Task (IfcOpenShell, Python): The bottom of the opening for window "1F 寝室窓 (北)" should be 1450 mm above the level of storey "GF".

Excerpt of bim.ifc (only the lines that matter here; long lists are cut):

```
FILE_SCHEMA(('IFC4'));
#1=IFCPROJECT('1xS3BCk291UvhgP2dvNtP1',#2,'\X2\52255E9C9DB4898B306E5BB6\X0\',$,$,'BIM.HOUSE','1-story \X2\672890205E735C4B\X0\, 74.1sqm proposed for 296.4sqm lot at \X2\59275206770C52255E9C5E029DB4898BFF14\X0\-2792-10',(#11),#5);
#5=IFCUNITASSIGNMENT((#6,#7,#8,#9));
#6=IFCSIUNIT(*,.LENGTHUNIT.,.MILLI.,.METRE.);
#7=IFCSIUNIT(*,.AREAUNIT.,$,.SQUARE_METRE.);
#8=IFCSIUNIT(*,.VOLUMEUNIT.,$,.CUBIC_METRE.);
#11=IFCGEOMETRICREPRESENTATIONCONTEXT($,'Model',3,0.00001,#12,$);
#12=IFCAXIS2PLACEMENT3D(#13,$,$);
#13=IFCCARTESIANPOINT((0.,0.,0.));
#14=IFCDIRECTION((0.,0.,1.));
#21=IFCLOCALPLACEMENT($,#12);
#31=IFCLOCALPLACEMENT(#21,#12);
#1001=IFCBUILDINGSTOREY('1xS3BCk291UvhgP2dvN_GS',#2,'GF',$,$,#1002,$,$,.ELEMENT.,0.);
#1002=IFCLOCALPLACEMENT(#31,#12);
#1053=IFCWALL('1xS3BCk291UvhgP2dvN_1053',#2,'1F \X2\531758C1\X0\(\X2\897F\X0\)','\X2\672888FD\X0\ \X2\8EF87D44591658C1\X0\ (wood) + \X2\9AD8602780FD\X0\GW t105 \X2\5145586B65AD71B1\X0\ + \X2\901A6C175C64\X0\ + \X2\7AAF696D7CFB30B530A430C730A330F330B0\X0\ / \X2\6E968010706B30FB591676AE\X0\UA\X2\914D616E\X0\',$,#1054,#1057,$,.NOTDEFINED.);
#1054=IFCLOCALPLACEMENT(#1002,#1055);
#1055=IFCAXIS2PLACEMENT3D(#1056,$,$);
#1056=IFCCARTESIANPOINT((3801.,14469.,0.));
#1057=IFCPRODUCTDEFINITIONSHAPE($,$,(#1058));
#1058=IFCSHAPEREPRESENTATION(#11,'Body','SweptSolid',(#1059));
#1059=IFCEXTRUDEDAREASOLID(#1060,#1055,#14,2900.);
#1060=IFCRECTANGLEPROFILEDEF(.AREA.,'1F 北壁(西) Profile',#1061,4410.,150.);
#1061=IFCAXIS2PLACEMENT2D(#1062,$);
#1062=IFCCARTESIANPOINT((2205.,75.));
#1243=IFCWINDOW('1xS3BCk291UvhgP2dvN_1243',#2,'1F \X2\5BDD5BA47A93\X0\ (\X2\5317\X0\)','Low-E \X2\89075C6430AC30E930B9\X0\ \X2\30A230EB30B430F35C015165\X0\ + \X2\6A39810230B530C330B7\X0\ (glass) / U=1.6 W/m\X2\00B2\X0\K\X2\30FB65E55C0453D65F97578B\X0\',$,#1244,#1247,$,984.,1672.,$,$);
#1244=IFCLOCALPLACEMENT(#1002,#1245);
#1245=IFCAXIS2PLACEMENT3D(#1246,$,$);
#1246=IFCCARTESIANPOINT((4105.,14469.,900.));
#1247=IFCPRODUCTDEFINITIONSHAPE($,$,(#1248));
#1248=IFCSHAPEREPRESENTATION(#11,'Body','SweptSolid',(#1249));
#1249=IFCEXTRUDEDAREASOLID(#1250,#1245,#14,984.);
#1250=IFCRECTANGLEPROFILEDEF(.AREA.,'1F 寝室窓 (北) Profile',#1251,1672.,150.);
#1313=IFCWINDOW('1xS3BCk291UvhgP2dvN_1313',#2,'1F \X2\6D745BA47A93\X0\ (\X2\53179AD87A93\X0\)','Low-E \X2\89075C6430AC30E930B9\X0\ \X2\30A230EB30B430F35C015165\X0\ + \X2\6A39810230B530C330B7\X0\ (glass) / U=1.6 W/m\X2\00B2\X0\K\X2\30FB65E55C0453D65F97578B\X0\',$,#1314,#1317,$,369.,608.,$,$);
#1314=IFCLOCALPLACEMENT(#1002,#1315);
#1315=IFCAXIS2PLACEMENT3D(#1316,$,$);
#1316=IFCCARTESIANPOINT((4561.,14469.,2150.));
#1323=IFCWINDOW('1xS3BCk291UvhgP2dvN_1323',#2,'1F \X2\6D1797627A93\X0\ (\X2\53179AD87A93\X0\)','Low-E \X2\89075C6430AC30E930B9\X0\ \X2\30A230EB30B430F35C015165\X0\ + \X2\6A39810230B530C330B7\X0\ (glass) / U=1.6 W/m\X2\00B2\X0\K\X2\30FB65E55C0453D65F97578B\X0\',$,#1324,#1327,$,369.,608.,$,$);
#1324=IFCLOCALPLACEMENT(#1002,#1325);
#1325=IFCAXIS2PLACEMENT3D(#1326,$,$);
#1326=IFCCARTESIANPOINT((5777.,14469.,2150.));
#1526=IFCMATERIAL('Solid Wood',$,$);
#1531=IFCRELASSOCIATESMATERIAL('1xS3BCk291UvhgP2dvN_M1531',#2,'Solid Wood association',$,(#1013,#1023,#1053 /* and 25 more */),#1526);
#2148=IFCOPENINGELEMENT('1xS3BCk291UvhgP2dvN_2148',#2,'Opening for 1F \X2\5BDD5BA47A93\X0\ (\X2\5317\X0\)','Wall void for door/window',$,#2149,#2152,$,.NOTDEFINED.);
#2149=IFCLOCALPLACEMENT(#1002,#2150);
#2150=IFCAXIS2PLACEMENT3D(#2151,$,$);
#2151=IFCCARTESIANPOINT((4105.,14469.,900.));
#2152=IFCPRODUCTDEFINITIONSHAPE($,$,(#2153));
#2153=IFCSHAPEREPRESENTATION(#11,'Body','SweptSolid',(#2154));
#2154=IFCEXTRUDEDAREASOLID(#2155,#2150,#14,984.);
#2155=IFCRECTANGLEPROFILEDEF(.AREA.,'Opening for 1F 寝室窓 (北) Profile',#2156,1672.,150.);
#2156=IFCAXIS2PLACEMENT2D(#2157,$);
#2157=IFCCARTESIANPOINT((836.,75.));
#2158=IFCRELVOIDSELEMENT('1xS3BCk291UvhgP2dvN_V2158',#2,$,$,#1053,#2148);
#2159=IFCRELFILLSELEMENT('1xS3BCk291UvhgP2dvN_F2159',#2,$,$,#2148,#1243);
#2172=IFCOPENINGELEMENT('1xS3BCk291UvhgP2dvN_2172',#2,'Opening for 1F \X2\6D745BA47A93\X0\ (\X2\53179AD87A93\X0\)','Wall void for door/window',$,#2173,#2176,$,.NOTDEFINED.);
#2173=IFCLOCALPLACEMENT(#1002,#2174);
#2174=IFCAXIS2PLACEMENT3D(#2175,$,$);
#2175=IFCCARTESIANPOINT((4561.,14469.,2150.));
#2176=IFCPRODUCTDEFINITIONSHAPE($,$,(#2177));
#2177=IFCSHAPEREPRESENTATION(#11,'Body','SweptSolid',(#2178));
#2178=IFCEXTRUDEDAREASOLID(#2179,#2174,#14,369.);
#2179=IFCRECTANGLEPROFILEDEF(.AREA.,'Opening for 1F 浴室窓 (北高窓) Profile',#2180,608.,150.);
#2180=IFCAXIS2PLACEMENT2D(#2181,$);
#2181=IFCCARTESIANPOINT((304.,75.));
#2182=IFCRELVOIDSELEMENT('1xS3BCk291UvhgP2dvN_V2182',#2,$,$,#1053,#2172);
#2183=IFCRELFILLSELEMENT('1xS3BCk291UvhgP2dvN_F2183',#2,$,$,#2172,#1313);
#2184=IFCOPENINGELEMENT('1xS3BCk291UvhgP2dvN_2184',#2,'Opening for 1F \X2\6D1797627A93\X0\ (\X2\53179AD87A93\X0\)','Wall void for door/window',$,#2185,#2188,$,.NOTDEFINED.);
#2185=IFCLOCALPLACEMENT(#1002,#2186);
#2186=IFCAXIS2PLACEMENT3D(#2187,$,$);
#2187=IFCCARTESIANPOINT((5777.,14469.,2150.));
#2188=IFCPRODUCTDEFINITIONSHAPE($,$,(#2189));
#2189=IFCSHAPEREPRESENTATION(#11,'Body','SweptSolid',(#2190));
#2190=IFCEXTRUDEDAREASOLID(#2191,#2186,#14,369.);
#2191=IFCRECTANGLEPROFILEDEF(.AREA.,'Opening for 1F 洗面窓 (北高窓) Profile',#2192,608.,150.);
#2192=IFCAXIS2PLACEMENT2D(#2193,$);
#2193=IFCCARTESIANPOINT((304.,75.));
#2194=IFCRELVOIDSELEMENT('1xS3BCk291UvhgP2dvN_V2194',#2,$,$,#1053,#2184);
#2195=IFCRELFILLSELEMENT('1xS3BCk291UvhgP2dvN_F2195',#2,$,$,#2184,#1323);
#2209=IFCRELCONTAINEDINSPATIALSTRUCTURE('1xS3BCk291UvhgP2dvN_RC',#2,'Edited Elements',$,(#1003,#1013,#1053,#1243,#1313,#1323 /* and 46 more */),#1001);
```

```python
import numpy as np
import ifcopenshell
import ifcopenshell.api.geometry
import ifcopenshell.geom
import ifcopenshell.util.element
import ifcopenshell.util.placement
import ifcopenshell.util.shape
import ifcopenshell.util.unit

model = ifcopenshell.open("bim.ifc")
unit_scale = ifcopenshell.util.unit.calculate_unit_scale(model)

window = model.by_id(1243)
opening = window.FillsVoids[0].RelatingOpeningElement
storey = ifcopenshell.util.element.get_container(window, ifc_class="IfcBuildingStorey")
level = ifcopenshell.util.placement.get_local_placement(storey.ObjectPlacement)[2, 3]

# The opening's origin need not be at the sill, so measure its lowest point.
shape = ifcopenshell.geom.create_shape(ifcopenshell.geom.settings(), opening)
bottom = ifcopenshell.util.shape.get_shape_bottom_elevation(shape, shape.geometry) / unit_scale
dz = level + 1450.0 - bottom

shift = np.array([0.0, 0.0, dz])
# The window is not placed relative to its opening, so move both.
for product in (opening, window):
    matrix = ifcopenshell.util.placement.get_local_placement(product.ObjectPlacement)
    matrix[:3, 3] += shift
    ifcopenshell.api.geometry.edit_object_placement(model, product=product, matrix=matrix, is_si=False)

print(f"moved by {dz * unit_scale:+.3f} m")

model.write("bim-out.ifc")
```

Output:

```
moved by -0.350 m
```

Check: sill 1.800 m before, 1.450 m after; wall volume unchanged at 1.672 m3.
